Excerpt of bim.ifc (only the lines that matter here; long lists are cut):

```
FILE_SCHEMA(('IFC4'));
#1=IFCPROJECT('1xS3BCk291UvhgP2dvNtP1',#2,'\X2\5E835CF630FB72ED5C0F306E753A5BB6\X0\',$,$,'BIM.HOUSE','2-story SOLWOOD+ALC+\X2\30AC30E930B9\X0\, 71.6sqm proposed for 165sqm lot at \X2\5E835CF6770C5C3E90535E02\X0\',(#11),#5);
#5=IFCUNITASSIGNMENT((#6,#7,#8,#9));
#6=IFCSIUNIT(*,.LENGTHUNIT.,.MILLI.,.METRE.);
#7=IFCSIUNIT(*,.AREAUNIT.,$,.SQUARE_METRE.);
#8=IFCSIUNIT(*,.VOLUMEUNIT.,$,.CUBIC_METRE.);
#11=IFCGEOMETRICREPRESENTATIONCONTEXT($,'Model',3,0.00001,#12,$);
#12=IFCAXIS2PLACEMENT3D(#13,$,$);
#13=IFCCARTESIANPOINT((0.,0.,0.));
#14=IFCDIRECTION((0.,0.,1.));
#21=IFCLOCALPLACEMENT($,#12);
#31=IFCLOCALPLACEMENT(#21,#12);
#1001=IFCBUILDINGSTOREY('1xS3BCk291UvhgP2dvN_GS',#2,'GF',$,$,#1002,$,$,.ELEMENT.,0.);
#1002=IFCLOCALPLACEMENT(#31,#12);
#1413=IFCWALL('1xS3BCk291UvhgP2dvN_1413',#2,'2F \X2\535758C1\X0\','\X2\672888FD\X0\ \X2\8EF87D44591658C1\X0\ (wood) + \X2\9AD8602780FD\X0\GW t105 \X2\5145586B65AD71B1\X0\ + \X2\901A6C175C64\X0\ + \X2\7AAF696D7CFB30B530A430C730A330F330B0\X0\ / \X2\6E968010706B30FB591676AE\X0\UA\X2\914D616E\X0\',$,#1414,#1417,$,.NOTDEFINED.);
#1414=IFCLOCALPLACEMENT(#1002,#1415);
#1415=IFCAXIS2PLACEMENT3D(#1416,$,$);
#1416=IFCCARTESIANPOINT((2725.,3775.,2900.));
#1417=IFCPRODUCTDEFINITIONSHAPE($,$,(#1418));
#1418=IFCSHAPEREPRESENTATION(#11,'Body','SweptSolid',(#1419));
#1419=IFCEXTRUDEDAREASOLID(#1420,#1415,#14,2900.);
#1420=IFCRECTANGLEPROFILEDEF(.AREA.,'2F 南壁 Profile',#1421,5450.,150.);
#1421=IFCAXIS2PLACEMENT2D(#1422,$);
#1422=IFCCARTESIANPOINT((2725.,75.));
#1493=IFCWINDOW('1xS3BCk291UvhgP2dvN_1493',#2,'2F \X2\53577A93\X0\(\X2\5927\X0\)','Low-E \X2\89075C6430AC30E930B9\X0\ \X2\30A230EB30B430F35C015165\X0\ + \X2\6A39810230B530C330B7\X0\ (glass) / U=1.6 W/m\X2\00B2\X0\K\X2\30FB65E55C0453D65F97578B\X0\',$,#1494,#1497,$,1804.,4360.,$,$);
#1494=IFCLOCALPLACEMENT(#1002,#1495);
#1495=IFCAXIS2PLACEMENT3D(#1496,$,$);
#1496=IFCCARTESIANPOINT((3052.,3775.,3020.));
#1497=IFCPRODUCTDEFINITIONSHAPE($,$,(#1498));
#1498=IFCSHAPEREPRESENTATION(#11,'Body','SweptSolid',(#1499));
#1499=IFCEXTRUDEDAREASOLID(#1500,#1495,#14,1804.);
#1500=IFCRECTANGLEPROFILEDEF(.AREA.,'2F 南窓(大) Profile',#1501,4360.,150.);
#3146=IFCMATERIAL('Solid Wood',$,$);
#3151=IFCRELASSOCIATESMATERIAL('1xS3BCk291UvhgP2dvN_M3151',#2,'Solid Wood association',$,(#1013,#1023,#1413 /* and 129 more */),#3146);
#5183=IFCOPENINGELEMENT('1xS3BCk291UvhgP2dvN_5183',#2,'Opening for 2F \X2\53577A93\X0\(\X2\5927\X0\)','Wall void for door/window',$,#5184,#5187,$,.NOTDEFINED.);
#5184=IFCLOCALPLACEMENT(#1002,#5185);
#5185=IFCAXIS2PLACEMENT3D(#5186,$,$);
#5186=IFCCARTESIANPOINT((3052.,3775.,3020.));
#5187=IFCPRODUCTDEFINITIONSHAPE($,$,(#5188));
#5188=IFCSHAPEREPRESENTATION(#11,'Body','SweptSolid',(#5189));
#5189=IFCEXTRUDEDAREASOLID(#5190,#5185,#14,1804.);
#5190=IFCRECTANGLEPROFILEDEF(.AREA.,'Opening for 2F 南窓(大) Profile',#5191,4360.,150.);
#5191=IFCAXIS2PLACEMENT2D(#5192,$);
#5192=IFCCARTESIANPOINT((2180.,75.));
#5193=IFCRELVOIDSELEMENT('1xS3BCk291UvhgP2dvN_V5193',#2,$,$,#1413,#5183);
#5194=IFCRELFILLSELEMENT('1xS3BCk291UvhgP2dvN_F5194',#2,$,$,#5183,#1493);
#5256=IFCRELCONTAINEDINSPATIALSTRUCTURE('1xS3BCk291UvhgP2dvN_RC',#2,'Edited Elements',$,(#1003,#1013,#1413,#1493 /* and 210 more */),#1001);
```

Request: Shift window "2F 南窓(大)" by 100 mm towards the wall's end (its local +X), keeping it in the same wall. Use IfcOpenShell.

```python
import ifcopenshell
import ifcopenshell.api.geometry
import ifcopenshell.util.placement
import ifcopenshell.util.unit

model = ifcopenshell.open("bim.ifc")
unit_scale = ifcopenshell.util.unit.calculate_unit_scale(model)

window = model.by_guid("1xS3BCk291UvhgP2dvN_1493")
opening = window.FillsVoids[0].RelatingOpeningElement
wall = opening.VoidsElements[0].RelatingBuildingElement

wall_matrix = ifcopenshell.util.placement.get_local_placement(wall.ObjectPlacement)
shift = wall_matrix[:3, 0] * 0.1 / unit_scale
before = ifcopenshell.util.placement.get_local_placement(window.ObjectPlacement)[:3, 3].copy()

# The window is not placed relative to its opening, so move both.
for product in (opening, window):
    matrix = ifcopenshell.util.placement.get_local_placement(product.ObjectPlacement)
    matrix[:3, 3] += shift
    ifcopenshell.api.geometry.edit_object_placement(model, product=product, matrix=matrix, is_si=False)

after = ifcopenshell.util.placement.get_local_placement(window.ObjectPlacement)[:3, 3]
print("window moved by", (after - before).round(3) + 0.0)

model.write("bim_v2.ifc")
```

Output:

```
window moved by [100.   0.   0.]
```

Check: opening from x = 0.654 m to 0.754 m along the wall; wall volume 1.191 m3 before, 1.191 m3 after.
